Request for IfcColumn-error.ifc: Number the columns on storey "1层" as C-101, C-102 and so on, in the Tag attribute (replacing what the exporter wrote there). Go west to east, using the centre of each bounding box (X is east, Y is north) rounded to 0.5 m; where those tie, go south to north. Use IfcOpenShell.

First a look at what the model holds.

```python
import ifcopenshell
import ifcopenshell.util.element
import ifcopenshell.util.placement

model = ifcopenshell.open("IfcColumn-error.ifc")
print(model.schema)
storey = next(s for s in model.by_type("IfcBuildingStorey") if s.Name == "1层")
columns = [e for e in ifcopenshell.util.element.get_decomposition(storey) if e.is_a("IfcColumn")]
for e in sorted(columns, key=lambda e: e.id()):
    origin = ifcopenshell.util.placement.get_local_placement(e.ObjectPlacement)[:3, 3]
    print(e.id(), e.Tag, e.Name, origin.round(2) + 0.0, sep=" | ")
```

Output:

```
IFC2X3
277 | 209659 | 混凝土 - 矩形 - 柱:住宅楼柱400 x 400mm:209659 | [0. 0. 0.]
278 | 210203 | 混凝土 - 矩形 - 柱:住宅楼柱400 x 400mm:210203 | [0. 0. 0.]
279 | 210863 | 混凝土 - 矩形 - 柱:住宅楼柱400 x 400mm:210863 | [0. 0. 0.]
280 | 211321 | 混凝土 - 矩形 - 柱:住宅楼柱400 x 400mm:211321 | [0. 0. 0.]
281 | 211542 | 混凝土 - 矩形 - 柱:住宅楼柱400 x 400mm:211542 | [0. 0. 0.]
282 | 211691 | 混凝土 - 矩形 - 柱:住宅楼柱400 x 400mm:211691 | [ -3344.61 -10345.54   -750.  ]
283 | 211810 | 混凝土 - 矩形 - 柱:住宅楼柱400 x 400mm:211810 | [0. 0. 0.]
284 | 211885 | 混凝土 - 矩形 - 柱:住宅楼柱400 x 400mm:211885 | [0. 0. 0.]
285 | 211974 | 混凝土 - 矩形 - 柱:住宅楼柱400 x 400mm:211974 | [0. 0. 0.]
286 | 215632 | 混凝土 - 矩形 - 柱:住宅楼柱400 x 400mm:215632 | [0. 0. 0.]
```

```python
import ifcopenshell
import ifcopenshell.geom
import ifcopenshell.util.element
import ifcopenshell.util.shape

model = ifcopenshell.open("IfcColumn-error.ifc")
settings = ifcopenshell.geom.settings()
settings.set("use-world-coords", True)


def centre(element):
    shape = ifcopenshell.geom.create_shape(settings, element)
    return ifcopenshell.util.shape.get_bbox_centroid(shape.geometry)


storey = next(s for s in model.by_type("IfcBuildingStorey") if s.Name == "1层")
columns = [e for e in ifcopenshell.util.element.get_decomposition(storey) if e.is_a("IfcColumn")]

# Insertion points can sit at a corner or the storey origin, so sort by the geometry (in metres).
centres = {e: centre(e) for e in columns}
columns.sort(key=lambda e: (round(centres[e][0] / 0.5), centres[e][1]))

for i, e in enumerate(columns, start=1):
    number = f"C-1{i:02d}"
    e.Tag = number
    print(e.id(), number)

model.write("IfcColumn-error-out.ifc")
```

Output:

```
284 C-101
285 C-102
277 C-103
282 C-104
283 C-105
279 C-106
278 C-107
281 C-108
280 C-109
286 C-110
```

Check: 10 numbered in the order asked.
